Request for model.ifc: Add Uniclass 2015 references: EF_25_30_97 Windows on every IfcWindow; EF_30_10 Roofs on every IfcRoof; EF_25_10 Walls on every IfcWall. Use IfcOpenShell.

First a look at what the model holds.

```python
import ifcopenshell

model = ifcopenshell.open("model.ifc")
print(model.schema)
print("classifications:", [c.Name for c in model.by_type("IfcClassification")])
for ifc_class in ("IfcDoor", "IfcRoof", "IfcStair", "IfcWall", "IfcWindow"):
    print(ifc_class, len(model.by_type(ifc_class)))
```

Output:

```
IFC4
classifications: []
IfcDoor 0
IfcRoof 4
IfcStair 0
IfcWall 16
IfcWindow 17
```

```python
import ifcopenshell
import ifcopenshell.api.classification

model = ifcopenshell.open("model.ifc")

system = ifcopenshell.api.classification.add_classification(model, classification="Uniclass 2015")

codes = {
    "IfcWindow": ("EF_25_30_97", "Windows"),
    "IfcRoof": ("EF_30_10", "Roofs"),
    "IfcWall": ("EF_25_10", "Walls"),
}
for ifc_class, (code, name) in codes.items():
    products = model.by_type(ifc_class)
    ifcopenshell.api.classification.add_reference(
        model, products=products, classification=system, identification=code, name=name
    )
    print(code, len(products))

model.write("model-out.ifc")
```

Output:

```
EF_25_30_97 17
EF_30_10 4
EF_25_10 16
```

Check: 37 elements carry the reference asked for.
